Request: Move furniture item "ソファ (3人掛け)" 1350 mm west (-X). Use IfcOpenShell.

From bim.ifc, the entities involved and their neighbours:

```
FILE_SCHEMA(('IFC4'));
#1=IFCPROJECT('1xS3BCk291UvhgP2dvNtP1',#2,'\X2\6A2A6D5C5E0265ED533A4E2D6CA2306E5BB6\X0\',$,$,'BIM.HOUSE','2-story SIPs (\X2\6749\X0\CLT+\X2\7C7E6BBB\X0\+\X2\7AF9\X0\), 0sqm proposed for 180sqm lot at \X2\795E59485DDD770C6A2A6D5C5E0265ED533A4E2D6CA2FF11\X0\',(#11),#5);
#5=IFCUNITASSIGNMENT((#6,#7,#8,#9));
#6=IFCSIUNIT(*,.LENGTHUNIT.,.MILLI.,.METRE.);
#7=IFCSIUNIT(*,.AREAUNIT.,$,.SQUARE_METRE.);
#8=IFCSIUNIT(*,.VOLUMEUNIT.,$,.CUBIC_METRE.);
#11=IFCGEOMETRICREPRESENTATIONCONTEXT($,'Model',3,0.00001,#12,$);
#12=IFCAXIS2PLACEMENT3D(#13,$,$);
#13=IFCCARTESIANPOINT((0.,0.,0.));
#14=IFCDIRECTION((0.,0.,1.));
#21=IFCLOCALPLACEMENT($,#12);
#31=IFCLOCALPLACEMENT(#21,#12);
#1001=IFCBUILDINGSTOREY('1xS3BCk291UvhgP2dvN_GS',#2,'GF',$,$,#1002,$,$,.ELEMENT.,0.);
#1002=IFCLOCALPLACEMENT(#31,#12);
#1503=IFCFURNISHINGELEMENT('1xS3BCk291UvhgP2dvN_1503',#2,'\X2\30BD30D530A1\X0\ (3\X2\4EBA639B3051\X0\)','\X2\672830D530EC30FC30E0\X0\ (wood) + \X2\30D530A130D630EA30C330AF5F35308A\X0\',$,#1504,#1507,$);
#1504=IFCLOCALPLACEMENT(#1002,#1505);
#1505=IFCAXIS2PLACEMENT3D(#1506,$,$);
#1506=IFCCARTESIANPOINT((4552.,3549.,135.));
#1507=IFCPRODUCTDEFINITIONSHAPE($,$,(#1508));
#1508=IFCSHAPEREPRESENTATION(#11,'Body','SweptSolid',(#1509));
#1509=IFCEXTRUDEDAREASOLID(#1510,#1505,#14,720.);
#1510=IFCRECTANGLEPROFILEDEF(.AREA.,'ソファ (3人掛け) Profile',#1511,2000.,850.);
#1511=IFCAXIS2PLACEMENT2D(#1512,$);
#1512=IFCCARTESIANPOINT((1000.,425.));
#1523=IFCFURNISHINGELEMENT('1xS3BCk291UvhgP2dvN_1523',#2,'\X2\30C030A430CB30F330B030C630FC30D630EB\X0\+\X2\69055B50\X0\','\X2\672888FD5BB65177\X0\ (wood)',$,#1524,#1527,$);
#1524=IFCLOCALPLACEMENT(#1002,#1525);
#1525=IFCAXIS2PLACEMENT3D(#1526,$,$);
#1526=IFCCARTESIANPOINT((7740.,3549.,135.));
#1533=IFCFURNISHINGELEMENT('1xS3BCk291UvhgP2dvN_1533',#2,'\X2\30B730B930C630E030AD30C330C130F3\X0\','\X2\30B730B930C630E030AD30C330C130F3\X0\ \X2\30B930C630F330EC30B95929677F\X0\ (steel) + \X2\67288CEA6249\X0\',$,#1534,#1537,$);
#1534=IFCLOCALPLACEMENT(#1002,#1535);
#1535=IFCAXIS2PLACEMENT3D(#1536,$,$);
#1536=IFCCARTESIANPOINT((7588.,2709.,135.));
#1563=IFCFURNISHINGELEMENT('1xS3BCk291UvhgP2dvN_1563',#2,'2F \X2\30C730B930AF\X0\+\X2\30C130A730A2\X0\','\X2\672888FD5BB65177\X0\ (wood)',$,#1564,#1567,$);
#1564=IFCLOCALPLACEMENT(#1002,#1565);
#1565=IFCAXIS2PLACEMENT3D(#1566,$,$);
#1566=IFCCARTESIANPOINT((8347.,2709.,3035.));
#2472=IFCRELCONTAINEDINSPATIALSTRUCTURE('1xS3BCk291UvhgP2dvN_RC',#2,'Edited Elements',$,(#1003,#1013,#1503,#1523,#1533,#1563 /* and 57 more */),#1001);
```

```python
import ifcopenshell
import ifcopenshell.api.geometry
import ifcopenshell.util.placement
import ifcopenshell.util.unit

model = ifcopenshell.open("bim.ifc")
unit_scale = ifcopenshell.util.unit.calculate_unit_scale(model)

item = model.by_guid("1xS3BCk291UvhgP2dvN_1503")
matrix = ifcopenshell.util.placement.get_local_placement(item.ObjectPlacement)
matrix[0, 3] -= 1.35 / unit_scale
ifcopenshell.api.geometry.edit_object_placement(model, product=item, matrix=matrix, is_si=False)

print(ifcopenshell.util.placement.get_local_placement(item.ObjectPlacement).round(3) + 0.0)

model.write("bim_v2.ifc")
```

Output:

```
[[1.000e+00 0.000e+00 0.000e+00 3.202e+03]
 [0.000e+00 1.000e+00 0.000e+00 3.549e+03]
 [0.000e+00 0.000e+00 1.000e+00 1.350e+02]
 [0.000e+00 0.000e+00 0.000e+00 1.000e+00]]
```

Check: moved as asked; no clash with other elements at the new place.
